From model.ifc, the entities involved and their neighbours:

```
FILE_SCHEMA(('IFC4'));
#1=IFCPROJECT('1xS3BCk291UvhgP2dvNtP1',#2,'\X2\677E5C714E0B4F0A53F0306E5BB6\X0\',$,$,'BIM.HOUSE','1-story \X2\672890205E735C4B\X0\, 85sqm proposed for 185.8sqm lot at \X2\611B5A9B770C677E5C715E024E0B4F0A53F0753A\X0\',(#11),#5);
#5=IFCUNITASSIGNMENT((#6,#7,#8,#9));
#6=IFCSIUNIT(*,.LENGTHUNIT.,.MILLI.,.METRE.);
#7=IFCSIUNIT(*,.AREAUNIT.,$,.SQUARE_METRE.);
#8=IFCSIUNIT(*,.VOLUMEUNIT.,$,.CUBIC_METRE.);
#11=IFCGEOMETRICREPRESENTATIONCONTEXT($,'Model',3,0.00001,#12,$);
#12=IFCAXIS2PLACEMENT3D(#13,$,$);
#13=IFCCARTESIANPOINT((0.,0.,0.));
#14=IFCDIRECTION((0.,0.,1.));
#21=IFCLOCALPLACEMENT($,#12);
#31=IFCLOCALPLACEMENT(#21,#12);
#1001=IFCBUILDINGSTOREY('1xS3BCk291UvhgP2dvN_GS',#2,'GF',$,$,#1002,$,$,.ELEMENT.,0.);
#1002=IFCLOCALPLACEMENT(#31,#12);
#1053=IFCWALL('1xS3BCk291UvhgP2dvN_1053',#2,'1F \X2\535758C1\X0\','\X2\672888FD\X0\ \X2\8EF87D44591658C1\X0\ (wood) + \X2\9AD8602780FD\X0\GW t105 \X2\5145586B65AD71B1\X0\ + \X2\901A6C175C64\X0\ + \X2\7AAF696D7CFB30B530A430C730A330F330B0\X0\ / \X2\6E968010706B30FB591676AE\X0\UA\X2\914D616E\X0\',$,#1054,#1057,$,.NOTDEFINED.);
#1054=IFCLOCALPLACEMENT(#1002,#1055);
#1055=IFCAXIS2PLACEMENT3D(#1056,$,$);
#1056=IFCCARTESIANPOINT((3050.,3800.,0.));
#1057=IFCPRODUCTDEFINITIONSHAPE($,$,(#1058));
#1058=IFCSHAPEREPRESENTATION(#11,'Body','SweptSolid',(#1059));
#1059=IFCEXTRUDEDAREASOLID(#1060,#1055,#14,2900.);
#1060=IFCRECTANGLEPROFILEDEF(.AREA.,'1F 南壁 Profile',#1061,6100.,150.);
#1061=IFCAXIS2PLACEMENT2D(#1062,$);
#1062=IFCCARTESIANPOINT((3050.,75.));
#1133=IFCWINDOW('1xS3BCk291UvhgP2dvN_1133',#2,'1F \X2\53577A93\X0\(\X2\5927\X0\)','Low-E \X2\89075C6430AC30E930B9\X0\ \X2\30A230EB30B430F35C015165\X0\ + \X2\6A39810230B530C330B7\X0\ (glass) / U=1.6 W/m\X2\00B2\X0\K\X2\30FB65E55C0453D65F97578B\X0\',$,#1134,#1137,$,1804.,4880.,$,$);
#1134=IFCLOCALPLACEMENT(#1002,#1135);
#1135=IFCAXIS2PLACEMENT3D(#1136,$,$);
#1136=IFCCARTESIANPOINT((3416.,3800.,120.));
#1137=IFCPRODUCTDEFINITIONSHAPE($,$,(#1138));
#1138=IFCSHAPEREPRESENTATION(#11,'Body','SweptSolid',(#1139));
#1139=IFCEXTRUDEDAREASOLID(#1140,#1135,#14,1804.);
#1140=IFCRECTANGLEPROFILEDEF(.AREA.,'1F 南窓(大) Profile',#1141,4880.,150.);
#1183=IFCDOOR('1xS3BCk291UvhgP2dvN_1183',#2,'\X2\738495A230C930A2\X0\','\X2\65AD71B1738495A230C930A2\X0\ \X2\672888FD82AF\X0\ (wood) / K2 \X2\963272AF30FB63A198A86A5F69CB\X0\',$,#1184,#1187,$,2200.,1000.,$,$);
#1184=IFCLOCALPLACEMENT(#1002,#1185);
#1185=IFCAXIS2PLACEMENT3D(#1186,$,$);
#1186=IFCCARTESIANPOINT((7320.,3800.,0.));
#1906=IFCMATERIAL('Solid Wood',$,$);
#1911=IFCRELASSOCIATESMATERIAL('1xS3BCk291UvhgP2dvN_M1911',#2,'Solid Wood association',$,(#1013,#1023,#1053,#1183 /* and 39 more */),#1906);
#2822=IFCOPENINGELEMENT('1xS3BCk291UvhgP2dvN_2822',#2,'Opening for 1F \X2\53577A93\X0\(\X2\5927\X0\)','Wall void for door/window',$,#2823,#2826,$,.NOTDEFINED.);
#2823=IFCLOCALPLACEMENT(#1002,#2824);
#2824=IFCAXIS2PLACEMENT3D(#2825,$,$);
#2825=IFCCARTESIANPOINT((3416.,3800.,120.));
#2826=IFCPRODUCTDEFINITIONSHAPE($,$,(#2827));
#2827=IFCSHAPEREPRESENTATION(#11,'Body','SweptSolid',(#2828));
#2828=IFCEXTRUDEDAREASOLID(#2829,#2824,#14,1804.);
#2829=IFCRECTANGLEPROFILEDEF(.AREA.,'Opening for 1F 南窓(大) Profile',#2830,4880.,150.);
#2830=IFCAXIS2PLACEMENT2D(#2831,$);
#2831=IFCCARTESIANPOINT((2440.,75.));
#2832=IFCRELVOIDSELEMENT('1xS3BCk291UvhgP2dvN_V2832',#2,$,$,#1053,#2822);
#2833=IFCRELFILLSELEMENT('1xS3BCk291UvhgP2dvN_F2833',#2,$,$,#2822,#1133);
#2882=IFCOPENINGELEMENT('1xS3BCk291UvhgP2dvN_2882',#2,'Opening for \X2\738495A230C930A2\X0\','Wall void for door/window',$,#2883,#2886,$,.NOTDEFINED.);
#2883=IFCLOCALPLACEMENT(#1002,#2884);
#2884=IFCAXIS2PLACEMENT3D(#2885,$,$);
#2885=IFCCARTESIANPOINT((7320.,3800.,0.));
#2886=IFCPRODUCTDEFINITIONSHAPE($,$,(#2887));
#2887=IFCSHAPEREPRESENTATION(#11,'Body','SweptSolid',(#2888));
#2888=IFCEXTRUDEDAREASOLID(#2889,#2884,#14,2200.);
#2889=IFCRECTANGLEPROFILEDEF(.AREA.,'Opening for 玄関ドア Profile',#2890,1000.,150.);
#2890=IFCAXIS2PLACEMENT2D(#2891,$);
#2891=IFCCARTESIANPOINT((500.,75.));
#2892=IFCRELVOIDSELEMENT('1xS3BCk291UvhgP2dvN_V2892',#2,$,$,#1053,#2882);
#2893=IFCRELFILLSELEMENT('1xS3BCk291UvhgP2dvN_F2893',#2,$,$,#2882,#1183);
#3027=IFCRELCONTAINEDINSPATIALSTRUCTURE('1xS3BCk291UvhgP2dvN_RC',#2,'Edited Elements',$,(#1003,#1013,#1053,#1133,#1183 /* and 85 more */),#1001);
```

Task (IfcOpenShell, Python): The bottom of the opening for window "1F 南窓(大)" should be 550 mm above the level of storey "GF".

```python
import numpy as np
import ifcopenshell
import ifcopenshell.api.geometry
import ifcopenshell.geom
import ifcopenshell.util.element
import ifcopenshell.util.placement
import ifcopenshell.util.shape
import ifcopenshell.util.unit

model = ifcopenshell.open("model.ifc")
unit_scale = ifcopenshell.util.unit.calculate_unit_scale(model)

window = model.by_guid("1xS3BCk291UvhgP2dvN_1133")
opening = window.FillsVoids[0].RelatingOpeningElement
storey = ifcopenshell.util.element.get_container(window, ifc_class="IfcBuildingStorey")
level = ifcopenshell.util.placement.get_local_placement(storey.ObjectPlacement)[2, 3]

# The opening's origin need not be at the sill, so measure its lowest point.
shape = ifcopenshell.geom.create_shape(ifcopenshell.geom.settings(), opening)
bottom = ifcopenshell.util.shape.get_shape_bottom_elevation(shape, shape.geometry) / unit_scale
dz = level + 0.55 / unit_scale - bottom

shift = np.array([0.0, 0.0, dz])
# The window is not placed relative to its opening, so move both.
for product in (opening, window):
    matrix = ifcopenshell.util.placement.get_local_placement(product.ObjectPlacement)
    matrix[:3, 3] += shift
    ifcopenshell.api.geometry.edit_object_placement(model, product=product, matrix=matrix, is_si=False)

print(f"moved by {dz * unit_scale:+.3f} m")

model.write("model-out.ifc")
```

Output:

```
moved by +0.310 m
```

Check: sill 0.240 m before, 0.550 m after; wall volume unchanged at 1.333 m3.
